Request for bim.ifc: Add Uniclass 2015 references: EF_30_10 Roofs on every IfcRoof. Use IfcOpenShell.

First a look at what the model holds.

```python
import ifcopenshell

model = ifcopenshell.open("bim.ifc")
print(model.schema)
print("classifications:", [c.Name for c in model.by_type("IfcClassification")])
for ifc_class in ("IfcDoor", "IfcRoof", "IfcStair", "IfcWall", "IfcWindow"):
    print(ifc_class, len(model.by_type(ifc_class)))
```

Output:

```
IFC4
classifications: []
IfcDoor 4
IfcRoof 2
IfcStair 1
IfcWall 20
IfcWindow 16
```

```python
import ifcopenshell
import ifcopenshell.api.classification

model = ifcopenshell.open("bim.ifc")

system = ifcopenshell.api.classification.add_classification(model, classification="Uniclass 2015")

codes = {
    "IfcRoof": ("EF_30_10", "Roofs"),
}
for ifc_class, (code, name) in codes.items():
    products = model.by_type(ifc_class)
    ifcopenshell.api.classification.add_reference(
        model, products=products, classification=system, identification=code, name=name
    )
    print(code, len(products))

model.write("bim_updated.ifc")
```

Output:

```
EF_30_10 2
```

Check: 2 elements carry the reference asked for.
